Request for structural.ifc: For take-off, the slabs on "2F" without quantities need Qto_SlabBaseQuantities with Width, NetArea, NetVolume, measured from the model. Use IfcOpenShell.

First a look at what the model holds.

```python
import ifcopenshell
import ifcopenshell.util.element
import ifcopenshell.util.unit

model = ifcopenshell.open("structural.ifc")
print(model.schema)
for unit_type in ("LENGTHUNIT", "AREAUNIT", "VOLUMEUNIT"):
    print(unit_type, ifcopenshell.util.unit.calculate_unit_scale(model, unit_type))
storey = next(s for s in model.by_type("IfcBuildingStorey") if s.Name == "2F")
slabs = [e for e in ifcopenshell.util.element.get_decomposition(storey) if e.is_a("IfcSlab")]
for e in sorted(slabs, key=lambda e: e.id()):
    print(e.id(), e.is_a(), e.Name, list(ifcopenshell.util.element.get_psets(e, qtos_only=True)), sep=" | ")
```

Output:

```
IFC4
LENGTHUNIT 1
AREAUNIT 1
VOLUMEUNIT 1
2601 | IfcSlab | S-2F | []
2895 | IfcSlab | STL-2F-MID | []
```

```python
import ifcopenshell
import ifcopenshell.api.pset
import ifcopenshell.geom
import ifcopenshell.util.element
import ifcopenshell.util.shape
import ifcopenshell.util.unit

model = ifcopenshell.open("structural.ifc")
unit_scale = ifcopenshell.util.unit.calculate_unit_scale(model)
area_scale = ifcopenshell.util.unit.calculate_unit_scale(model, "AREAUNIT")
volume_scale = ifcopenshell.util.unit.calculate_unit_scale(model, "VOLUMEUNIT")
settings = ifcopenshell.geom.settings()

storey = next(s for s in model.by_type("IfcBuildingStorey") if s.Name == "2F")
slabs = [e for e in ifcopenshell.util.element.get_decomposition(storey) if e.is_a("IfcSlab")]

for e in sorted(slabs, key=lambda e: e.id()):
    if ifcopenshell.util.element.get_psets(e, qtos_only=True, should_inherit=False):
        continue
    # Geometry comes back in metres, in the element's own axes.
    shape = ifcopenshell.geom.create_shape(settings, e)
    values = {
        "Width": ifcopenshell.util.shape.get_z(shape.geometry) / unit_scale,
        "NetArea": ifcopenshell.util.shape.get_footprint_area(shape.geometry) / area_scale,
        "NetVolume": ifcopenshell.util.shape.get_volume(shape.geometry) / volume_scale,
    }
    qto = ifcopenshell.api.pset.add_qto(model, product=e, name="Qto_SlabBaseQuantities")
    ifcopenshell.api.pset.edit_qto(model, qto=qto, properties=values)
    print(e.id(), {k: round(v, 3) for k, v in values.items()})

model.write("structural_updated.ifc")
```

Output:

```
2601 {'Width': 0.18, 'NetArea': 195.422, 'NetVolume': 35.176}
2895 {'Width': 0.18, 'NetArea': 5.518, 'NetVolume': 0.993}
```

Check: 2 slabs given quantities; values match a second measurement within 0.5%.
